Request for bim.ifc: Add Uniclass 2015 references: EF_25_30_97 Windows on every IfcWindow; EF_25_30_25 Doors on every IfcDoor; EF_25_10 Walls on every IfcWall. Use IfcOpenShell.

First a look at what the model holds.

```python
import ifcopenshell

model = ifcopenshell.open("bim.ifc")
print(model.schema)
print("classifications:", [c.Name for c in model.by_type("IfcClassification")])
for ifc_class in ("IfcDoor", "IfcRoof", "IfcStair", "IfcWall", "IfcWindow"):
    print(ifc_class, len(model.by_type(ifc_class)))
```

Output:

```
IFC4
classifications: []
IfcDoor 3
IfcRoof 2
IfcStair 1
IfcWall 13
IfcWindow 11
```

```python
import ifcopenshell
import ifcopenshell.api.classification

model = ifcopenshell.open("bim.ifc")

system = ifcopenshell.api.classification.add_classification(model, classification="Uniclass 2015")

codes = {
    "IfcWindow": ("EF_25_30_97", "Windows"),
    "IfcDoor": ("EF_25_30_25", "Doors"),
    "IfcWall": ("EF_25_10", "Walls"),
}
for ifc_class, (code, name) in codes.items():
    products = model.by_type(ifc_class)
    ifcopenshell.api.classification.add_reference(
        model, products=products, classification=system, identification=code, name=name
    )
    print(code, len(products))

model.write("bim-out.ifc")
```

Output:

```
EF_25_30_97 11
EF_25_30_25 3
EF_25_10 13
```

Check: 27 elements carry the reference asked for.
